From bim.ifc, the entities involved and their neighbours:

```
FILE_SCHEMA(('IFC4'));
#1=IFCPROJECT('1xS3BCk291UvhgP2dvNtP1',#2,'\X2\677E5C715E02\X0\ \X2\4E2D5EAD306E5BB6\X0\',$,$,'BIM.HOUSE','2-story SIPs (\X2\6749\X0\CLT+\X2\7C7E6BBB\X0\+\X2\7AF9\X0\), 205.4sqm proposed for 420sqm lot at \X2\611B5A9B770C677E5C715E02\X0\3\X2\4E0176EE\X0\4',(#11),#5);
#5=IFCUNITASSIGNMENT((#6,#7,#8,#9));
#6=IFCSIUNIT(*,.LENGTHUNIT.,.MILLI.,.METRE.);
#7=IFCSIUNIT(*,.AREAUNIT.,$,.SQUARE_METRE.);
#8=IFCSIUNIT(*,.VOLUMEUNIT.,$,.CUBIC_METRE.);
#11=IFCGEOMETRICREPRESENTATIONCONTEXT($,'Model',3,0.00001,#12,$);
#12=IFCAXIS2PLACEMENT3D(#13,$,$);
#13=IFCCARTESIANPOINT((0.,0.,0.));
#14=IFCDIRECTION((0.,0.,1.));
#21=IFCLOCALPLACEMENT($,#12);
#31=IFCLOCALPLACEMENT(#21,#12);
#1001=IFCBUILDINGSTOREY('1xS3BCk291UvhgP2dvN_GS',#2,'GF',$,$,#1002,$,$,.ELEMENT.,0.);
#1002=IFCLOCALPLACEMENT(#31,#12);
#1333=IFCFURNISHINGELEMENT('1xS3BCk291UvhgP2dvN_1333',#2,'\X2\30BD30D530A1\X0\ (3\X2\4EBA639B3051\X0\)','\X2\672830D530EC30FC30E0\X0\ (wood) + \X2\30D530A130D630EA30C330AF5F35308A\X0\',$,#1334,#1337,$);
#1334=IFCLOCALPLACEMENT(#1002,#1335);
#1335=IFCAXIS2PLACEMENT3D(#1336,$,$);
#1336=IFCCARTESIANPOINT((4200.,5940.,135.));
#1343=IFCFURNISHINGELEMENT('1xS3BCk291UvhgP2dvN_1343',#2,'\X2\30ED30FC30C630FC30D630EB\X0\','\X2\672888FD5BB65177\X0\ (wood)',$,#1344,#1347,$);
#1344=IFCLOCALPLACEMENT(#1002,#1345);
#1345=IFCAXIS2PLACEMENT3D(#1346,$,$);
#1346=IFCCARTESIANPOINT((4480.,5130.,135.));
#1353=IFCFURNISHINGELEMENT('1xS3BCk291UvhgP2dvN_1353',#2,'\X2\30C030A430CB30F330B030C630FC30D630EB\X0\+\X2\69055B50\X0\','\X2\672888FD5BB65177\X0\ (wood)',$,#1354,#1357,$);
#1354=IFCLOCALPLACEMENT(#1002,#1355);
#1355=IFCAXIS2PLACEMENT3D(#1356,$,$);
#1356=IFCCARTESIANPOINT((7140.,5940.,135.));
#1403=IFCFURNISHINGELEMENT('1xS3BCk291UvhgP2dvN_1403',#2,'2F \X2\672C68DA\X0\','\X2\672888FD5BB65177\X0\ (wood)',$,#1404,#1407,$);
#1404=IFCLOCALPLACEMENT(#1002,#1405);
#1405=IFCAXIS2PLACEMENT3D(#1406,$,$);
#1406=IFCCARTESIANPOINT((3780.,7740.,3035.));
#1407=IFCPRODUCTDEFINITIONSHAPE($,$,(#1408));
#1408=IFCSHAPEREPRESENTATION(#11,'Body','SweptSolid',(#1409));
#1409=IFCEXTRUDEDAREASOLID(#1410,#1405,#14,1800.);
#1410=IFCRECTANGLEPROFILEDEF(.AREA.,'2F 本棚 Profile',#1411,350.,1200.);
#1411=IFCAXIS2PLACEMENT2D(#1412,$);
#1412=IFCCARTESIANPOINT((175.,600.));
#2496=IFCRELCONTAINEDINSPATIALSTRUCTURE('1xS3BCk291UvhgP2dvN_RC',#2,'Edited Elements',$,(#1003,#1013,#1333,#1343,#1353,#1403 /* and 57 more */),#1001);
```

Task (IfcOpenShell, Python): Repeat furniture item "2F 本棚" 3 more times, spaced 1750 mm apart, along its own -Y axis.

```python
import ifcopenshell
import ifcopenshell.api.geometry
import ifcopenshell.api.root
import ifcopenshell.util.element
import ifcopenshell.util.placement
import ifcopenshell.util.unit

model = ifcopenshell.open("bim.ifc")
unit_scale = ifcopenshell.util.unit.calculate_unit_scale(model)


def reuse_history(source, copy):
    """copy_class also copies each property set's owner history, people and application; keep the originals."""
    for rel in copy.IsDefinedBy:
        if rel.is_a("IfcRelDefinesByProperties") and (history := rel.RelatingPropertyDefinition.OwnerHistory):
            rel.RelatingPropertyDefinition.OwnerHistory = source.OwnerHistory
            ifcopenshell.util.element.remove_deep2(model, history)


source = model.by_guid("1xS3BCk291UvhgP2dvN_1403")
base = ifcopenshell.util.placement.get_local_placement(source.ObjectPlacement)
step = -base[:3, 1] * 1.75 / unit_scale

for i in range(1, 4):
    copy = ifcopenshell.api.root.copy_class(model, product=source)
    copy.Representation = ifcopenshell.util.element.copy_deep(
        model, source.Representation, exclude=["IfcGeometricRepresentationContext", "IfcRepresentationMap"]
    )
    reuse_history(source, copy)
    matrix = base.copy()
    matrix[:3, 3] += i * step
    print("added at", matrix[:3, 3].round(3) + 0.0)
    ifcopenshell.api.geometry.edit_object_placement(model, product=copy, matrix=matrix, is_si=False)

model.write("bim_rev.ifc")
```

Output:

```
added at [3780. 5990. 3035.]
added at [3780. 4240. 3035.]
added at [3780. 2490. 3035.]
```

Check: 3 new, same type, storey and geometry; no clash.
